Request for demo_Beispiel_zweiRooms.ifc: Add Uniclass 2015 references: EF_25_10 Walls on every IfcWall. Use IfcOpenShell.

First a look at what the model holds.

```python
import ifcopenshell

model = ifcopenshell.open("demo_Beispiel_zweiRooms.ifc")
print(model.schema)
print("classifications:", [c.Name for c in model.by_type("IfcClassification")])
for ifc_class in ("IfcDoor", "IfcRoof", "IfcStair", "IfcWall", "IfcWindow"):
    print(ifc_class, len(model.by_type(ifc_class)))
```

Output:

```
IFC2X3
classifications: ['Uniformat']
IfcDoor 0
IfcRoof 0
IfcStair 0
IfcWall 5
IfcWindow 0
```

```python
import ifcopenshell
import ifcopenshell.api.classification

model = ifcopenshell.open("demo_Beispiel_zweiRooms.ifc")

# IFC2X3 requires Source and Edition and has no link from the project to the system.
system = model.create_entity("IfcClassification", Source="NBS", Edition="2015", Name="Uniclass 2015")

codes = {
    "IfcWall": ("EF_25_10", "Walls"),
}
for ifc_class, (code, name) in codes.items():
    products = model.by_type(ifc_class)
    ifcopenshell.api.classification.add_reference(
        model, products=products, classification=system, identification=code, name=name
    )
    print(code, len(products))

model.write("demo_Beispiel_zweiRooms_edited.ifc")
```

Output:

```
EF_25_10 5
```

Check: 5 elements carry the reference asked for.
